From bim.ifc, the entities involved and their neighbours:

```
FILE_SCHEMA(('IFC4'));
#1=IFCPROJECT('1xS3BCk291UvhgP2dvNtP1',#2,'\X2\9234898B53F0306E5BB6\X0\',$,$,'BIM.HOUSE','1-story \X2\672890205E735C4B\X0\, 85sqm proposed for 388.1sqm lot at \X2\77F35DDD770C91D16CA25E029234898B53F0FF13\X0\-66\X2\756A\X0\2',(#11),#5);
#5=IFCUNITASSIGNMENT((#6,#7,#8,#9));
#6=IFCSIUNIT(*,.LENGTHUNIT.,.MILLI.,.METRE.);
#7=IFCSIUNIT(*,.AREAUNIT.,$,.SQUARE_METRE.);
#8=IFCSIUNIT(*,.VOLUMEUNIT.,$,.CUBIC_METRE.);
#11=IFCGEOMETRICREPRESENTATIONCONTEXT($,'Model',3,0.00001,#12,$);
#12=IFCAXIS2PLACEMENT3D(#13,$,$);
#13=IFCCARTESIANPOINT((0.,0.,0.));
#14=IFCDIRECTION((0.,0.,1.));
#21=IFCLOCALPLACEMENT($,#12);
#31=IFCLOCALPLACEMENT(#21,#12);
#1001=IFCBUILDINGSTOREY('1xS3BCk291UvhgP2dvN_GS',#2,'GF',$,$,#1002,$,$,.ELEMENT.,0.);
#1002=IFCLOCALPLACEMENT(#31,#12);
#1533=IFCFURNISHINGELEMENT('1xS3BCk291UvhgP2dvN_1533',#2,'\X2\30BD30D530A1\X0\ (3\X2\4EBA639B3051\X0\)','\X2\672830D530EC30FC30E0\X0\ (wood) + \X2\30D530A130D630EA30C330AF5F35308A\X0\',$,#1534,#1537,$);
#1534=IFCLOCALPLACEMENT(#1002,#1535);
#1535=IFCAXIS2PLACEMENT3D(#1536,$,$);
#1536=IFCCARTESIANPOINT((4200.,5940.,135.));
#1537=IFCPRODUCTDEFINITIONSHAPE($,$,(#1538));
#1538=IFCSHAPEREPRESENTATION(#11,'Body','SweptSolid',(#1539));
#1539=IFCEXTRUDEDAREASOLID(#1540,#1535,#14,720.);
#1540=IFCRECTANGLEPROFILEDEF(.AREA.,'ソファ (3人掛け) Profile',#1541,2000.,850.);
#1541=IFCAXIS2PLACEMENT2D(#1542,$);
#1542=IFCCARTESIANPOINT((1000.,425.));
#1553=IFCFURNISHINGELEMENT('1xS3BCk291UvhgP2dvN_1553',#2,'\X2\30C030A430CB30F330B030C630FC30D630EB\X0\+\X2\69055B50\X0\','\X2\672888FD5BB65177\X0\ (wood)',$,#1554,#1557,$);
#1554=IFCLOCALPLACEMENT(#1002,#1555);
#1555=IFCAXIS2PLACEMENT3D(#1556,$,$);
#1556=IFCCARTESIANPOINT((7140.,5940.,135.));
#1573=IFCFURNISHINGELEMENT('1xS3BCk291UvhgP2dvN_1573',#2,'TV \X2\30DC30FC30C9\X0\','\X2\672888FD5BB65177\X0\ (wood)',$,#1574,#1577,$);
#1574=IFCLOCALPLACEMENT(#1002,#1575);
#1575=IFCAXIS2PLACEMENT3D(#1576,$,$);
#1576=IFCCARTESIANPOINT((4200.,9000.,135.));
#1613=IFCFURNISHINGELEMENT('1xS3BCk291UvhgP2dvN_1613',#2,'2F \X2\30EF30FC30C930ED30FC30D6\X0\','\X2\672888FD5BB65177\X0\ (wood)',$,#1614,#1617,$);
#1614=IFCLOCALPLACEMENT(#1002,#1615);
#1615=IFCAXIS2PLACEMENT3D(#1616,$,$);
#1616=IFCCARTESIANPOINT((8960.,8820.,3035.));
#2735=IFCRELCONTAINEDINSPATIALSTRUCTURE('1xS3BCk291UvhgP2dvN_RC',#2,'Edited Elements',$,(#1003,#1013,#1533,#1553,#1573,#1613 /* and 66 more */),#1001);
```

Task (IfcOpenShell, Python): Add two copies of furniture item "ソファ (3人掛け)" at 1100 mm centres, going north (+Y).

```python
import numpy as np
import ifcopenshell
import ifcopenshell.api.geometry
import ifcopenshell.api.root
import ifcopenshell.util.element
import ifcopenshell.util.placement

model = ifcopenshell.open("bim.ifc")


def reuse_history(source, copy):
    """copy_class also copies each property set's owner history, people and application; keep the originals."""
    for rel in copy.IsDefinedBy:
        if rel.is_a("IfcRelDefinesByProperties") and (history := rel.RelatingPropertyDefinition.OwnerHistory):
            rel.RelatingPropertyDefinition.OwnerHistory = source.OwnerHistory
            ifcopenshell.util.element.remove_deep2(model, history)


source = model.by_guid("1xS3BCk291UvhgP2dvN_1533")
base = ifcopenshell.util.placement.get_local_placement(source.ObjectPlacement)
step = np.array([0.0, 1.0, 0.0]) * 1100.0

for i in range(1, 3):
    copy = ifcopenshell.api.root.copy_class(model, product=source)
    copy.Representation = ifcopenshell.util.element.copy_deep(
        model, source.Representation, exclude=["IfcGeometricRepresentationContext", "IfcRepresentationMap"]
    )
    reuse_history(source, copy)
    matrix = base.copy()
    matrix[:3, 3] += i * step
    print("added at", matrix[:3, 3].round(3) + 0.0)
    ifcopenshell.api.geometry.edit_object_placement(model, product=copy, matrix=matrix, is_si=False)

model.write("bim_edited.ifc")
```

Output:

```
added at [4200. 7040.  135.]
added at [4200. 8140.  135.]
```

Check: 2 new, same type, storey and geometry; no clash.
